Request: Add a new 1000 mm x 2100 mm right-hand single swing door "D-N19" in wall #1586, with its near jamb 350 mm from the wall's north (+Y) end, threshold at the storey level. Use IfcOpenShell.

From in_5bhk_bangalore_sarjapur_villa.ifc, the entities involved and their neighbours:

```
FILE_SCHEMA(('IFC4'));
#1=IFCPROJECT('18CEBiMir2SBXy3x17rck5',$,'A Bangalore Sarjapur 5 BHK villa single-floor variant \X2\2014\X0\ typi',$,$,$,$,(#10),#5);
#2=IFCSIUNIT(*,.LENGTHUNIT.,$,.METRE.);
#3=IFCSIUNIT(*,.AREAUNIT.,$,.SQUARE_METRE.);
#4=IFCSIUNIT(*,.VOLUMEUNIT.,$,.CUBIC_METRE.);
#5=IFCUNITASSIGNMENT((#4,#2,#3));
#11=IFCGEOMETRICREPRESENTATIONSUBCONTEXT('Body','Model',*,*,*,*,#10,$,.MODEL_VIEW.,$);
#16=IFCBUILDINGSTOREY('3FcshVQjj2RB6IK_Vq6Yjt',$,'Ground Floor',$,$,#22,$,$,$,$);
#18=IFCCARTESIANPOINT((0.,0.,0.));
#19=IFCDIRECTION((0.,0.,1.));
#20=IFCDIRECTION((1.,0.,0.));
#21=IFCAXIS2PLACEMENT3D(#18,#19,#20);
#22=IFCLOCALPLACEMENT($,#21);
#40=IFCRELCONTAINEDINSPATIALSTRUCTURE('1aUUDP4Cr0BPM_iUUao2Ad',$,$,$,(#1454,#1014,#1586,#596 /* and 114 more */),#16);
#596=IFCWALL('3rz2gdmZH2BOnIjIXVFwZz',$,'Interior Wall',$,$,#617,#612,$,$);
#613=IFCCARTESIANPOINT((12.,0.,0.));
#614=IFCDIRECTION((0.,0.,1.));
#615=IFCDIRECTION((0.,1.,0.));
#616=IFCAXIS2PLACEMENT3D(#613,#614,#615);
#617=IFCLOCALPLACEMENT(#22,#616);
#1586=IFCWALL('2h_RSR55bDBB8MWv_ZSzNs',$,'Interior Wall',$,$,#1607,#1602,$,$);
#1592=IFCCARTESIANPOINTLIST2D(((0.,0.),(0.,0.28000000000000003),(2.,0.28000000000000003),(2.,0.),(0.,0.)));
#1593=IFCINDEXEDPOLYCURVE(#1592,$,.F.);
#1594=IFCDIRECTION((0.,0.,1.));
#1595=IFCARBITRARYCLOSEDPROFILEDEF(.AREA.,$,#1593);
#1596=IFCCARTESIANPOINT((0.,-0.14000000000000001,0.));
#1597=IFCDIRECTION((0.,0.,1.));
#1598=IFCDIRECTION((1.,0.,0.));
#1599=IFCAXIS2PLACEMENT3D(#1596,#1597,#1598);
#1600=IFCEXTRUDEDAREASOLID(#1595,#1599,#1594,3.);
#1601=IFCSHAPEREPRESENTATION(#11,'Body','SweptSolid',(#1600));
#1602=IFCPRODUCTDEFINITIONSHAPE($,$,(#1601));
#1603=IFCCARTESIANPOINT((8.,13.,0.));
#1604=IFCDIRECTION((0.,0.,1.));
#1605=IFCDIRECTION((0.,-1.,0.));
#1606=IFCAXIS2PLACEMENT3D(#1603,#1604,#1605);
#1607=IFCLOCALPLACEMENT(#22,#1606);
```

```python
import numpy as np
import ifcopenshell
import ifcopenshell.api.feature
import ifcopenshell.api.geometry
import ifcopenshell.api.root
import ifcopenshell.api.spatial
import ifcopenshell.geom
import ifcopenshell.util.element
import ifcopenshell.util.placement
import ifcopenshell.util.representation
import ifcopenshell.util.shape
import ifcopenshell.util.unit

model = ifcopenshell.open("in_5bhk_bangalore_sarjapur_villa.ifc")
unit_scale = ifcopenshell.util.unit.calculate_unit_scale(model)
settings = ifcopenshell.geom.settings()


def volume(element):
    """Net volume in cubic metres, openings subtracted."""
    shape = ifcopenshell.geom.create_shape(settings, element)
    return ifcopenshell.util.shape.get_volume(shape.geometry)


wall = model.by_guid("2h_RSR55bDBB8MWv_ZSzNs")
storey = ifcopenshell.util.element.get_container(wall, ifc_class="IfcBuildingStorey")
context = ifcopenshell.util.representation.get_context(model, "Model", "Body", "MODEL_VIEW")
before = volume(wall)

width, height, from_end, sill = 1, 2.1, 0.35, 0.0  # metres

# The wall runs along its own X axis, and the end named is its -X end.
wall_shape = ifcopenshell.geom.create_shape(settings, wall)
x, y, z = ifcopenshell.util.shape.get_vertices(wall_shape.geometry).T
start = x.min() + from_end
face, thickness = float(y.min()), float(y.max() - y.min())
wall_matrix = ifcopenshell.util.placement.get_local_placement(wall.ObjectPlacement)
level = ifcopenshell.util.placement.get_local_placement(storey.ObjectPlacement)[2, 3]


def in_wall(x, y):
    """Placement at x, y metres in the wall's axes, at sill height."""
    matrix = wall_matrix.copy()
    matrix[:, 3] = wall_matrix @ np.array([x / unit_scale, y / unit_scale, 0.0, 1.0])
    matrix[2, 3] = level + sill / unit_scale
    return matrix


# Opening: a box that overshoots both wall faces by 50 mm.
opening = ifcopenshell.api.root.create_entity(model, ifc_class="IfcOpeningElement", predefined_type="OPENING")
box = ifcopenshell.api.geometry.add_wall_representation(
    model, context=context, length=width, height=height, thickness=thickness + 0.1
)
ifcopenshell.api.geometry.assign_representation(model, product=opening, representation=box)
ifcopenshell.api.geometry.edit_object_placement(model, product=opening, matrix=in_wall(start, face - 0.05), is_si=False)
ifcopenshell.api.feature.add_feature(model, feature=opening, element=wall)

door = ifcopenshell.api.root.create_entity(model, ifc_class="IfcDoor", name="D-N19", predefined_type="DOOR")
door.OverallWidth, door.OverallHeight = width / unit_scale, height / unit_scale
door.OperationType = "SINGLE_SWING_RIGHT"
body = ifcopenshell.api.geometry.add_door_representation(
    model,
    context=context,
    overall_width=door.OverallWidth,
    overall_height=door.OverallHeight,
    operation_type="SINGLE_SWING_RIGHT",
    lining_properties={"LiningDepth": thickness / unit_scale, "ThresholdDepth": thickness / unit_scale},
)
ifcopenshell.api.geometry.assign_representation(model, product=door, representation=body)
ifcopenshell.api.spatial.assign_container(model, products=[door], relating_structure=storey)
ifcopenshell.api.feature.add_filling(model, opening=opening, element=door)

# The lining spans the wall, so the door starts at the wall face.
ifcopenshell.api.geometry.edit_object_placement(model, product=door, matrix=in_wall(start, face), is_si=False)

after = volume(wall)

print(f"wall volume {before:.3f} -> {after:.3f} m3")

model.write("in_5bhk_bangalore_sarjapur_villa_updated.ifc")
```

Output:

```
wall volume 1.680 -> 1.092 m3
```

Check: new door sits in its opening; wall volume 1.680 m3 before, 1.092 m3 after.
